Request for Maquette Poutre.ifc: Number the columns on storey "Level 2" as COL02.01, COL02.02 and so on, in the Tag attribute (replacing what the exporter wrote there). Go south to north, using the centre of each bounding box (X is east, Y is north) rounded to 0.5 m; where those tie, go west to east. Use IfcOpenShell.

First a look at what the model holds.

```python
import ifcopenshell
import ifcopenshell.util.element
import ifcopenshell.util.placement

model = ifcopenshell.open("Maquette Poutre.ifc")
print(model.schema)
storey = next(s for s in model.by_type("IfcBuildingStorey") if s.Name == "Level 2")
columns = [e for e in ifcopenshell.util.element.get_decomposition(storey) if e.is_a("IfcColumn")]
for e in sorted(columns, key=lambda e: e.id()):
    origin = ifcopenshell.util.placement.get_local_placement(e.ObjectPlacement)[:3, 3]
    print(e.id(), e.Tag, e.Name, origin.round(2) + 0.0, sep=" | ")
```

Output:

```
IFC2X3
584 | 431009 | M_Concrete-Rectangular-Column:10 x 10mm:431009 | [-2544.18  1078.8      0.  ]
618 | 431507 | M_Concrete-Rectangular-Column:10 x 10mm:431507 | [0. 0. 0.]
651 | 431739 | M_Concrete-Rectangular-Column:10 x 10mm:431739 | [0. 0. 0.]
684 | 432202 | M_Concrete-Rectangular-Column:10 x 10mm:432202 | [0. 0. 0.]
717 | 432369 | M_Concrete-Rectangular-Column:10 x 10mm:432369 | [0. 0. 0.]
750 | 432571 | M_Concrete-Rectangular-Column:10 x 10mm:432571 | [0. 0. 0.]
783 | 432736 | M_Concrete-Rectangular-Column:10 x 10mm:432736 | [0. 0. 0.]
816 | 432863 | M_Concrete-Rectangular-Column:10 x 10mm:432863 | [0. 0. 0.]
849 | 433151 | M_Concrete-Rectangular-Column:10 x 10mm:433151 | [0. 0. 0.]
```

```python
import ifcopenshell
import ifcopenshell.geom
import ifcopenshell.util.element
import ifcopenshell.util.shape

model = ifcopenshell.open("Maquette Poutre.ifc")
settings = ifcopenshell.geom.settings()
settings.set("use-world-coords", True)


def centre(element):
    shape = ifcopenshell.geom.create_shape(settings, element)
    return ifcopenshell.util.shape.get_bbox_centroid(shape.geometry)


storey = next(s for s in model.by_type("IfcBuildingStorey") if s.Name == "Level 2")
columns = [e for e in ifcopenshell.util.element.get_decomposition(storey) if e.is_a("IfcColumn")]

# Insertion points can sit at a corner or the storey origin, so sort by the geometry (in metres).
centres = {e: centre(e) for e in columns}
columns.sort(key=lambda e: (round(centres[e][1] / 0.5), centres[e][0]))

for i, e in enumerate(columns, start=1):
    number = f"COL02.{i:02d}"
    e.Tag = number
    print(e.id(), number)

model.write("Maquette Poutre-out.ifc")
```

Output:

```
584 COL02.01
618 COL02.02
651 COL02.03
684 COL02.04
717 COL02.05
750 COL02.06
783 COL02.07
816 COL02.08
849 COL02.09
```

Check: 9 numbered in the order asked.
